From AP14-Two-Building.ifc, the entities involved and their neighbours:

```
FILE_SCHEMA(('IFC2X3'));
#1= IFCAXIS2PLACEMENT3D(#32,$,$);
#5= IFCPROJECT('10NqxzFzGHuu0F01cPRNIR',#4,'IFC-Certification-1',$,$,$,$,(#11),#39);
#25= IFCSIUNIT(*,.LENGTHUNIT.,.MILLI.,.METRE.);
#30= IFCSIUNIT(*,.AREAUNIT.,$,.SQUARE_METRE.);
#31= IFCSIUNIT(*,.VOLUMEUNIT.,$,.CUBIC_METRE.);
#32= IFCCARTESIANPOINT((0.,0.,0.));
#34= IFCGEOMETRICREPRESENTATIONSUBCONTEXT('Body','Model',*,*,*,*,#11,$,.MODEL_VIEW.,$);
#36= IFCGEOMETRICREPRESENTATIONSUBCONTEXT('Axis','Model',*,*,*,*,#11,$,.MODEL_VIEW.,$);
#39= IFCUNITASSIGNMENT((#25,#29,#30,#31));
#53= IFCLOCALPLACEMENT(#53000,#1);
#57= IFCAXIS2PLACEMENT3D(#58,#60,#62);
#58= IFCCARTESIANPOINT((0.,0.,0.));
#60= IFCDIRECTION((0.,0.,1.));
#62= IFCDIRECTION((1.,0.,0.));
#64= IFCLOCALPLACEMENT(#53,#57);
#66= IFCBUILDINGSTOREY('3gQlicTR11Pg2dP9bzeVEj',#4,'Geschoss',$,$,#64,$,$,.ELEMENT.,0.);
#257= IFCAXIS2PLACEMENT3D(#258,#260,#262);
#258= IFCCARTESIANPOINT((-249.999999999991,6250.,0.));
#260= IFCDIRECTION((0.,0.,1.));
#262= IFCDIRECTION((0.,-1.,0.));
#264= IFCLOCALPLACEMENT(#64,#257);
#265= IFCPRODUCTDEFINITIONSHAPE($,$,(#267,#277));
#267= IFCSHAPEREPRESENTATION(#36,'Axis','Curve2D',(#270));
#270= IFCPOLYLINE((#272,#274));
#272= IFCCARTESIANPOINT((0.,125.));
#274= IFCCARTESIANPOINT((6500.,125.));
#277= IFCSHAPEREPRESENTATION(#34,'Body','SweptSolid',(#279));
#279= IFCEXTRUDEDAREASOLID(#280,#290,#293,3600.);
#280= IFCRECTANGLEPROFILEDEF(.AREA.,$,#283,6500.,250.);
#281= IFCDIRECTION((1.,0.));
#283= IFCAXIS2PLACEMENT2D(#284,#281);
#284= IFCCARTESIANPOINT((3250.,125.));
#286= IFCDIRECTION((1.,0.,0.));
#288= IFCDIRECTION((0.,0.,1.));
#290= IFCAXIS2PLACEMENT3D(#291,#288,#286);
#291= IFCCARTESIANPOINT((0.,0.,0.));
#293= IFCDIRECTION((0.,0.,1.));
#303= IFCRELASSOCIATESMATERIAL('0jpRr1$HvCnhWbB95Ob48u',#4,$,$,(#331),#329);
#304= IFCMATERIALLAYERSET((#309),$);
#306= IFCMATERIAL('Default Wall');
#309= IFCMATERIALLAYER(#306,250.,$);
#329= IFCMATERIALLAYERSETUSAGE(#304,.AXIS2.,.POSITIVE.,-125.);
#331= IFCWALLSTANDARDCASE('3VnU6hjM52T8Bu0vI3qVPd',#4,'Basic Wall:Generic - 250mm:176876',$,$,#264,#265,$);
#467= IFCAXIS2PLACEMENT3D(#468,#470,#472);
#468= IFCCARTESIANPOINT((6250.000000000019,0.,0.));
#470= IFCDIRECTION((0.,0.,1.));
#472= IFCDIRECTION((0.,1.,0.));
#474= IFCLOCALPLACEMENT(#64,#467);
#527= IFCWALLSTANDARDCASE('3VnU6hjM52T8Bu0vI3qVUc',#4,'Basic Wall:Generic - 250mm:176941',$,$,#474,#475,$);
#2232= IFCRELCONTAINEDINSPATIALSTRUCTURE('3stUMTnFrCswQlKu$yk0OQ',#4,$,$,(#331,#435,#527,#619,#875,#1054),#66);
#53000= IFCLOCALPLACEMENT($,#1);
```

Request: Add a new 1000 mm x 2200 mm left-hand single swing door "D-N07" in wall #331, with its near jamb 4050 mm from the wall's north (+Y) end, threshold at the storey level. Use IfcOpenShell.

```python
import numpy as np
import ifcopenshell
import ifcopenshell.api.feature
import ifcopenshell.api.geometry
import ifcopenshell.api.root
import ifcopenshell.api.spatial
import ifcopenshell.api.type
import ifcopenshell.geom
import ifcopenshell.util.element
import ifcopenshell.util.placement
import ifcopenshell.util.representation
import ifcopenshell.util.shape
import ifcopenshell.util.unit

model = ifcopenshell.open("AP14-Two-Building.ifc")
unit_scale = ifcopenshell.util.unit.calculate_unit_scale(model)
settings = ifcopenshell.geom.settings()


def volume(element):
    """Net volume in cubic metres, openings subtracted."""
    shape = ifcopenshell.geom.create_shape(settings, element)
    return ifcopenshell.util.shape.get_volume(shape.geometry)


wall = model.by_guid("3VnU6hjM52T8Bu0vI3qVPd")
storey = ifcopenshell.util.element.get_container(wall, ifc_class="IfcBuildingStorey")
context = ifcopenshell.util.representation.get_context(model, "Model", "Body", "MODEL_VIEW")
before = volume(wall)

width, height, from_end, sill = 1, 2.2, 4.05, 0.0  # metres

# The wall runs along its own X axis, and the end named is its -X end.
wall_shape = ifcopenshell.geom.create_shape(settings, wall)
x, y, z = ifcopenshell.util.shape.get_vertices(wall_shape.geometry).T
start = x.min() + from_end
face, thickness = float(y.min()), float(y.max() - y.min())
wall_matrix = ifcopenshell.util.placement.get_local_placement(wall.ObjectPlacement)
level = ifcopenshell.util.placement.get_local_placement(storey.ObjectPlacement)[2, 3]


def in_wall(x, y):
    """Placement at x, y metres in the wall's axes, at sill height."""
    matrix = wall_matrix.copy()
    matrix[:, 3] = wall_matrix @ np.array([x / unit_scale, y / unit_scale, 0.0, 1.0])
    matrix[2, 3] = level + sill / unit_scale
    return matrix


# Opening: a box that overshoots both wall faces by 50 mm.
opening = ifcopenshell.api.root.create_entity(model, ifc_class="IfcOpeningElement")
box = ifcopenshell.api.geometry.add_wall_representation(
    model, context=context, length=width, height=height, thickness=thickness + 0.1
)
ifcopenshell.api.geometry.assign_representation(model, product=opening, representation=box)
ifcopenshell.api.geometry.edit_object_placement(model, product=opening, matrix=in_wall(start, face - 0.05), is_si=False)
ifcopenshell.api.feature.add_feature(model, feature=opening, element=wall)

door = ifcopenshell.api.root.create_entity(model, ifc_class="IfcDoor", name="D-N07")
door.OverallWidth, door.OverallHeight = width / unit_scale, height / unit_scale
body = ifcopenshell.api.geometry.add_door_representation(
    model,
    context=context,
    overall_width=door.OverallWidth,
    overall_height=door.OverallHeight,
    operation_type="SINGLE_SWING_LEFT",
    lining_properties={"LiningDepth": thickness / unit_scale, "ThresholdDepth": thickness / unit_scale},
)
ifcopenshell.api.geometry.assign_representation(model, product=door, representation=body)
ifcopenshell.api.spatial.assign_container(model, products=[door], relating_structure=storey)
fills = ifcopenshell.api.feature.add_filling(model, opening=opening, element=door)
fills.OwnerHistory = door.OwnerHistory  # required in IFC2X3

# IFC2X3 keeps the operation on the door style.
style = ifcopenshell.api.root.create_entity(model, ifc_class="IfcDoorStyle", name="D-N07")
style.OperationType, style.ConstructionType = "SINGLE_SWING_LEFT", "NOTDEFINED"
style.ParameterTakesPrecedence = style.Sizeable = False
ifcopenshell.api.type.assign_type(model, related_objects=[door], relating_type=style)

# The lining spans the wall, so the door starts at the wall face.
ifcopenshell.api.geometry.edit_object_placement(model, product=door, matrix=in_wall(start, face), is_si=False)

after = volume(wall)

print(f"wall volume {before:.3f} -> {after:.3f} m3")

model.write("AP14-Two-Building_updated.ifc")
```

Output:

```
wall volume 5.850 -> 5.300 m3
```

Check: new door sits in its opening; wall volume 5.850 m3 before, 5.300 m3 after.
